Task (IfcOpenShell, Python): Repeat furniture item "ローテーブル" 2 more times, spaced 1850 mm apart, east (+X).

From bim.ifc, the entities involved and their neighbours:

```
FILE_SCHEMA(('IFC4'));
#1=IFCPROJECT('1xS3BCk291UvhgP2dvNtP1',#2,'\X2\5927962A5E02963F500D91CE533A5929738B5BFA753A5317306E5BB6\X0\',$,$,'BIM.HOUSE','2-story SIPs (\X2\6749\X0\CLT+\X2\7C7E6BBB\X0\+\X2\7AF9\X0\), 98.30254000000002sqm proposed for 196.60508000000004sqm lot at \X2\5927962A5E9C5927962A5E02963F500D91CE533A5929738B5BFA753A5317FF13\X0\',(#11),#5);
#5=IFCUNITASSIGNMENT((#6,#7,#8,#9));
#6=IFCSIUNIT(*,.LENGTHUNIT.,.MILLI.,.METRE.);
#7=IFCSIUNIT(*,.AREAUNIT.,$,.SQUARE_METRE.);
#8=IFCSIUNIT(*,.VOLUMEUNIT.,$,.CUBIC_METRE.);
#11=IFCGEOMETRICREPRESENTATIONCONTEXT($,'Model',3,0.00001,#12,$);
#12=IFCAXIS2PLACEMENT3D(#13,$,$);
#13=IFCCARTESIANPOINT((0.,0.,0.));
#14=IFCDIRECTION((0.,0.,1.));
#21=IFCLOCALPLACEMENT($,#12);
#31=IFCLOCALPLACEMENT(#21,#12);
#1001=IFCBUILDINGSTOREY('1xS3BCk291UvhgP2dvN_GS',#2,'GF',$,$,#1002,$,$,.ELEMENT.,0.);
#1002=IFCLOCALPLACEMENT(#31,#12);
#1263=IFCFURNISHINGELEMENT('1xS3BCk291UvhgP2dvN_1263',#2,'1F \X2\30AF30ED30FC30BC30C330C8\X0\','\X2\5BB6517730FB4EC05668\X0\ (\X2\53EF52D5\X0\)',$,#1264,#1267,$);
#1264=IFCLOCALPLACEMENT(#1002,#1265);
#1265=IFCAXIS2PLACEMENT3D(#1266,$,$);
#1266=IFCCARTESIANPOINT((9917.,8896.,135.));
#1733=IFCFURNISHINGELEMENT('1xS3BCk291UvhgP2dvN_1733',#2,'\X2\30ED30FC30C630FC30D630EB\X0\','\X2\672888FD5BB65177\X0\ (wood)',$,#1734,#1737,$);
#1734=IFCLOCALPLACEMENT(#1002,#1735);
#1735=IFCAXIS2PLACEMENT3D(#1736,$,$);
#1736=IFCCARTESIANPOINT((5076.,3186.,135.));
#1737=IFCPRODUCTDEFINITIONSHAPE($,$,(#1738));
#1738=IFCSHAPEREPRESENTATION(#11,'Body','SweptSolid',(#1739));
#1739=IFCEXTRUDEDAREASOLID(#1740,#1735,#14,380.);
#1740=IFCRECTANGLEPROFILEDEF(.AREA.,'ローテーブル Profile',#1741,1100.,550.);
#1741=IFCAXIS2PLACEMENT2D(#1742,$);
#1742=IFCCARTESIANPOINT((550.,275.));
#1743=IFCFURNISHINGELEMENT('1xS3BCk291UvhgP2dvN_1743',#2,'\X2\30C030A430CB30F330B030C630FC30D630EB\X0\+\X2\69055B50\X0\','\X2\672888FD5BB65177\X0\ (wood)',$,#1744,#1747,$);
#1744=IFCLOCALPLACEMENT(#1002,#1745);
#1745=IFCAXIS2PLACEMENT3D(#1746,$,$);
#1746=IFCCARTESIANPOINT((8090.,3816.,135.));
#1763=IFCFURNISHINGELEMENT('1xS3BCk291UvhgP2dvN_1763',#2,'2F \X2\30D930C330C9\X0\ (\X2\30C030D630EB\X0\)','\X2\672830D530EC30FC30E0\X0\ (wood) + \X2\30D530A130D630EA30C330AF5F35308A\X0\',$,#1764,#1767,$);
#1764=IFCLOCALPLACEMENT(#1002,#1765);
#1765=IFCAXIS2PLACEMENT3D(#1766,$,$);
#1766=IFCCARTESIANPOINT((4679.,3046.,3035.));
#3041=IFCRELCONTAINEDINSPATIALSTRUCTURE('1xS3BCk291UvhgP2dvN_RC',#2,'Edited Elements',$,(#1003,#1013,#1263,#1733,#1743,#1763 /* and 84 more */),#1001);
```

```python
import numpy as np
import ifcopenshell
import ifcopenshell.api.geometry
import ifcopenshell.api.root
import ifcopenshell.util.element
import ifcopenshell.util.placement
import ifcopenshell.util.unit

model = ifcopenshell.open("bim.ifc")
unit_scale = ifcopenshell.util.unit.calculate_unit_scale(model)


def reuse_history(source, copy):
    """copy_class also copies each property set's owner history, people and application; keep the originals."""
    for rel in copy.IsDefinedBy:
        if rel.is_a("IfcRelDefinesByProperties") and (history := rel.RelatingPropertyDefinition.OwnerHistory):
            rel.RelatingPropertyDefinition.OwnerHistory = source.OwnerHistory
            ifcopenshell.util.element.remove_deep2(model, history)


source = model.by_guid("1xS3BCk291UvhgP2dvN_1733")
base = ifcopenshell.util.placement.get_local_placement(source.ObjectPlacement)
step = np.array([1.0, 0.0, 0.0]) * 1.85 / unit_scale

for i in range(1, 3):
    copy = ifcopenshell.api.root.copy_class(model, product=source)
    copy.Representation = ifcopenshell.util.element.copy_deep(
        model, source.Representation, exclude=["IfcGeometricRepresentationContext", "IfcRepresentationMap"]
    )
    reuse_history(source, copy)
    matrix = base.copy()
    matrix[:3, 3] += i * step
    print("added at", matrix[:3, 3].round(3) + 0.0)
    ifcopenshell.api.geometry.edit_object_placement(model, product=copy, matrix=matrix, is_si=False)

model.write("bim-out.ifc")
```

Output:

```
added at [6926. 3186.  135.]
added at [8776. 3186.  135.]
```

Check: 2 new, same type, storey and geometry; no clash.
